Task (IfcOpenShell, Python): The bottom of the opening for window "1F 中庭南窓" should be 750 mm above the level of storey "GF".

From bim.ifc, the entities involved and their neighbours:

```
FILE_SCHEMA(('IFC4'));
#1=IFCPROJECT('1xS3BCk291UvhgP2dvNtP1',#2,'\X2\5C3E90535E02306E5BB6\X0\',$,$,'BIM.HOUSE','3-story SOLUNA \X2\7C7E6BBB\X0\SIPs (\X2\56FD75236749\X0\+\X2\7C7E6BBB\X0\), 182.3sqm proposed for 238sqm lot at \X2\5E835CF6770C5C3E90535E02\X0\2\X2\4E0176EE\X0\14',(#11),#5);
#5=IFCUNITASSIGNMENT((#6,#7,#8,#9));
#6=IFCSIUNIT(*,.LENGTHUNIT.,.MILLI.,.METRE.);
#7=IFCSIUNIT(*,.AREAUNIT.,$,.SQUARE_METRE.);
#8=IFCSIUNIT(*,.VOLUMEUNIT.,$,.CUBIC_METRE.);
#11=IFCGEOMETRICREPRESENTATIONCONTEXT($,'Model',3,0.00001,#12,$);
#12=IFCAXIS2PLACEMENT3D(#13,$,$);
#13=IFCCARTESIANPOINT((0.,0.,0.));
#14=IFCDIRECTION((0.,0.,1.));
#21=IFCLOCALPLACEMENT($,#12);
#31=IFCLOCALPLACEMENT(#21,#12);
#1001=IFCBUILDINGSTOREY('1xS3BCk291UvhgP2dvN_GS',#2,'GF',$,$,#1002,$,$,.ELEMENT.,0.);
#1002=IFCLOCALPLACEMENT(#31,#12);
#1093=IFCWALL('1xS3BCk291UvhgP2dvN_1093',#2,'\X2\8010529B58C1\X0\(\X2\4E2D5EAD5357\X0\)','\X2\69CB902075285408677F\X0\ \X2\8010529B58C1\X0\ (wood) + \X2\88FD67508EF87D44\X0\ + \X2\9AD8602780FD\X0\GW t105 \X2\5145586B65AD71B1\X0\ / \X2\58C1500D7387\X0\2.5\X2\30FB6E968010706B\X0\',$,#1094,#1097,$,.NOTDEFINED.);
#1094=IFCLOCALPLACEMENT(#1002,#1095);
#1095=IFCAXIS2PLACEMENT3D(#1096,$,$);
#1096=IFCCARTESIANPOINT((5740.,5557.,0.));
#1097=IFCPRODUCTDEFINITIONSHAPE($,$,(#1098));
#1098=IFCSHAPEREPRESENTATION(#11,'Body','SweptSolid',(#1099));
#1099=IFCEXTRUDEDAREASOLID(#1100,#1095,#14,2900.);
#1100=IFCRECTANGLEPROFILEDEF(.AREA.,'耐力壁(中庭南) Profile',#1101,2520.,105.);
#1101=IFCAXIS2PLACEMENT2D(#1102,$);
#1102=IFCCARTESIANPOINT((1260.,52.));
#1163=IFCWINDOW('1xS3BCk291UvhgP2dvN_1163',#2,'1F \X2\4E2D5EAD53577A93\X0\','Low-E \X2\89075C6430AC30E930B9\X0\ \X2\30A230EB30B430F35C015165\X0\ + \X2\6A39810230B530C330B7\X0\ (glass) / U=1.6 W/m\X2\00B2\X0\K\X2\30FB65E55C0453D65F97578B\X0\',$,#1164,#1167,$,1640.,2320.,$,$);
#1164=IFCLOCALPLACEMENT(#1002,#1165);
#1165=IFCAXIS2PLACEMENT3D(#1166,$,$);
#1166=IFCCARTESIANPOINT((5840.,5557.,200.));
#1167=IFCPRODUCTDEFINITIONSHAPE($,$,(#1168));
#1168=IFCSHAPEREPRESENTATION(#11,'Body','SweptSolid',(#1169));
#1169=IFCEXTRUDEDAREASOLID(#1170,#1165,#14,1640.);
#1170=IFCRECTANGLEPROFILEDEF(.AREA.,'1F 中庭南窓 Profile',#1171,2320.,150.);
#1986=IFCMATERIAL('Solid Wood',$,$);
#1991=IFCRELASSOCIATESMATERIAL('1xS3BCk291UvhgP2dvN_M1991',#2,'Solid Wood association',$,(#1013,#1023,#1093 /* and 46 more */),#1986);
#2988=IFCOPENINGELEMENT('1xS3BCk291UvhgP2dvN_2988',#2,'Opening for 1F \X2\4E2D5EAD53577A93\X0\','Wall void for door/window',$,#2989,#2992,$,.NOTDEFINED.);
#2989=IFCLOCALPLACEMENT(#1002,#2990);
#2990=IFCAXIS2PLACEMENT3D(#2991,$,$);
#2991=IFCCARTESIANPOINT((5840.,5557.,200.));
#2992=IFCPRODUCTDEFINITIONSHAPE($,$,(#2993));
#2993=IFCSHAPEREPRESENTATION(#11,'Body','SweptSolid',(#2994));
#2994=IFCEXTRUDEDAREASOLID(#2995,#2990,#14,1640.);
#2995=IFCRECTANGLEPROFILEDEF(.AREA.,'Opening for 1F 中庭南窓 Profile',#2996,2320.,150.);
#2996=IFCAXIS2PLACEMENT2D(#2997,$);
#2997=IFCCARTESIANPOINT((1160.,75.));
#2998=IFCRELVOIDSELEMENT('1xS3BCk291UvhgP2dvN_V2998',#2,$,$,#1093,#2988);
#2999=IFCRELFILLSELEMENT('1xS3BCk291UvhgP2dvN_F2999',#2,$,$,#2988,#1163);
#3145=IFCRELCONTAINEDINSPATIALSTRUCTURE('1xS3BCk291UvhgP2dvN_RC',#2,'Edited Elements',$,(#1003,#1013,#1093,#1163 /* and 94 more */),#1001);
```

```python
import numpy as np
import ifcopenshell
import ifcopenshell.api.geometry
import ifcopenshell.geom
import ifcopenshell.util.element
import ifcopenshell.util.placement
import ifcopenshell.util.shape
import ifcopenshell.util.unit

model = ifcopenshell.open("bim.ifc")
unit_scale = ifcopenshell.util.unit.calculate_unit_scale(model)

window = model.by_id(1163)
opening = window.FillsVoids[0].RelatingOpeningElement
storey = ifcopenshell.util.element.get_container(window, ifc_class="IfcBuildingStorey")
level = ifcopenshell.util.placement.get_local_placement(storey.ObjectPlacement)[2, 3]

# The opening's origin need not be at the sill, so measure its lowest point.
shape = ifcopenshell.geom.create_shape(ifcopenshell.geom.settings(), opening)
bottom = ifcopenshell.util.shape.get_shape_bottom_elevation(shape, shape.geometry) / unit_scale
dz = level + 750.0 - bottom

shift = np.array([0.0, 0.0, dz])
# The window is not placed relative to its opening, so move both.
for product in (opening, window):
    matrix = ifcopenshell.util.placement.get_local_placement(product.ObjectPlacement)
    matrix[:3, 3] += shift
    ifcopenshell.api.geometry.edit_object_placement(model, product=product, matrix=matrix, is_si=False)

print(f"moved by {dz * unit_scale:+.3f} m")

model.write("bim-out.ifc")
```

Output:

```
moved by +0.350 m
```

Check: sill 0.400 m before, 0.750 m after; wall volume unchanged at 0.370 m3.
